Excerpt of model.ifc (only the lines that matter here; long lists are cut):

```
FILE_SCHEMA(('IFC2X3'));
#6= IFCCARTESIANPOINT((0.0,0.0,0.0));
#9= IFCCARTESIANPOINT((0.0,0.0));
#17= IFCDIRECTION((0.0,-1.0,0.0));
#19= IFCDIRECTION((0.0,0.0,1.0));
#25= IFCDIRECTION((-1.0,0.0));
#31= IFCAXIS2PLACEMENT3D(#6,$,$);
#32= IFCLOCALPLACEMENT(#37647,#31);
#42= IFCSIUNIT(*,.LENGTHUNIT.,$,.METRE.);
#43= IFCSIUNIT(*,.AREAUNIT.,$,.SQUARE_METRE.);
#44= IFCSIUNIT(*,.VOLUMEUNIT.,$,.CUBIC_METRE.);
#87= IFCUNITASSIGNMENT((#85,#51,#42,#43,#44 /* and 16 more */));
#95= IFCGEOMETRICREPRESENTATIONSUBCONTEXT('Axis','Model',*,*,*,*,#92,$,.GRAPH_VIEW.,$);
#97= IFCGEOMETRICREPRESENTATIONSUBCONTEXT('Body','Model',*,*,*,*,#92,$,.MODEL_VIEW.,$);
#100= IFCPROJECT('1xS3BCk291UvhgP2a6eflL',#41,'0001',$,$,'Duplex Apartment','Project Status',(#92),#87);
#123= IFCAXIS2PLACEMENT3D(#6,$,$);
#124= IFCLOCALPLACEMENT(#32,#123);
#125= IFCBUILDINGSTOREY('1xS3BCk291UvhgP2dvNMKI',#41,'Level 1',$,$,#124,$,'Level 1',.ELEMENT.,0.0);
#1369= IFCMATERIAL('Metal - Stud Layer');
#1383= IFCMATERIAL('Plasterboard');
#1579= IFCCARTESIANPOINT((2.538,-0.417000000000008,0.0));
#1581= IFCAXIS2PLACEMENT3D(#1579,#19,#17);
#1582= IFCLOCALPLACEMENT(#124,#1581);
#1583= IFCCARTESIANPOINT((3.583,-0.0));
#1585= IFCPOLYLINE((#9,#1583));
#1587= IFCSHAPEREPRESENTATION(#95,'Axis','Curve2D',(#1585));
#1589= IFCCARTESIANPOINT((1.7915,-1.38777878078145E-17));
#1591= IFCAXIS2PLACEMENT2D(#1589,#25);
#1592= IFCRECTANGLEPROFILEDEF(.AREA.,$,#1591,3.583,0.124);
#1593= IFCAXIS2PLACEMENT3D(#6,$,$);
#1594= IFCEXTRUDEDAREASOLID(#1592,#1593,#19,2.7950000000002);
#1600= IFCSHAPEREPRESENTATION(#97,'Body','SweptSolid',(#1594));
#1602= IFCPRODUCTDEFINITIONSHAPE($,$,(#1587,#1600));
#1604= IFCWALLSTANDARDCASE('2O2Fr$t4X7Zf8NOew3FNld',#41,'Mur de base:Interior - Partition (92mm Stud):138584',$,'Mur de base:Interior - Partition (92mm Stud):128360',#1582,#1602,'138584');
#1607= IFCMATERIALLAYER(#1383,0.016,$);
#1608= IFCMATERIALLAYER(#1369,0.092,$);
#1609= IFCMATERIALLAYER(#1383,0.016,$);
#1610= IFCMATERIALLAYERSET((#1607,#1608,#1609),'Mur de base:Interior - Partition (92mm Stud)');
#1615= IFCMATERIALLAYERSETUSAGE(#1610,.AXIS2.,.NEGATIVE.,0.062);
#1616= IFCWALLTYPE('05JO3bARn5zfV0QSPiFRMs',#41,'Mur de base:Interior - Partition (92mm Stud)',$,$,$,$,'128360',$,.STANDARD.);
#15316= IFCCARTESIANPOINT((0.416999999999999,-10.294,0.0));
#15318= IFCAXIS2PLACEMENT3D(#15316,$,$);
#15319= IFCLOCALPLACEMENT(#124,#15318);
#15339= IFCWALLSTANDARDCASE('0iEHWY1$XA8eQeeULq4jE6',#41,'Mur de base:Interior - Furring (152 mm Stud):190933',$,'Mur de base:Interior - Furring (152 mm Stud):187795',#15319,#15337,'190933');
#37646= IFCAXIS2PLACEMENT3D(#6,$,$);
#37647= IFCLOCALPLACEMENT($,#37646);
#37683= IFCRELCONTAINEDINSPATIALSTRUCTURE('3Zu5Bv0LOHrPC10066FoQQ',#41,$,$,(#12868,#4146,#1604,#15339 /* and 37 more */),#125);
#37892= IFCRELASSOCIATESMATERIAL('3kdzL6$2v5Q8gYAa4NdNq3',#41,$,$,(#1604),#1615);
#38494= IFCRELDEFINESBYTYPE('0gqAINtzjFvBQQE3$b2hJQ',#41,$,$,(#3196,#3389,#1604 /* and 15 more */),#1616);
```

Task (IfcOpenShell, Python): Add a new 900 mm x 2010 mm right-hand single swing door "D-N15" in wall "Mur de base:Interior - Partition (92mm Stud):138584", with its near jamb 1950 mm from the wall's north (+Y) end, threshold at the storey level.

```python
import numpy as np
import ifcopenshell
import ifcopenshell.api.feature
import ifcopenshell.api.geometry
import ifcopenshell.api.root
import ifcopenshell.api.spatial
import ifcopenshell.api.type
import ifcopenshell.geom
import ifcopenshell.util.element
import ifcopenshell.util.placement
import ifcopenshell.util.representation
import ifcopenshell.util.shape
import ifcopenshell.util.unit

model = ifcopenshell.open("model.ifc")
unit_scale = ifcopenshell.util.unit.calculate_unit_scale(model)
settings = ifcopenshell.geom.settings()


def volume(element):
    """Net volume in cubic metres, openings subtracted."""
    shape = ifcopenshell.geom.create_shape(settings, element)
    return ifcopenshell.util.shape.get_volume(shape.geometry)


wall = model.by_guid("2O2Fr$t4X7Zf8NOew3FNld")
storey = ifcopenshell.util.element.get_container(wall, ifc_class="IfcBuildingStorey")
context = ifcopenshell.util.representation.get_context(model, "Model", "Body", "MODEL_VIEW")
before = volume(wall)

width, height, from_end, sill = 0.9, 2.01, 1.95, 0.0  # metres

# The wall runs along its own X axis, and the end named is its -X end.
wall_shape = ifcopenshell.geom.create_shape(settings, wall)
x, y, z = ifcopenshell.util.shape.get_vertices(wall_shape.geometry).T
start = x.min() + from_end
face, thickness = float(y.min()), float(y.max() - y.min())
wall_matrix = ifcopenshell.util.placement.get_local_placement(wall.ObjectPlacement)
level = ifcopenshell.util.placement.get_local_placement(storey.ObjectPlacement)[2, 3]


def in_wall(x, y):
    """Placement at x, y metres in the wall's axes, at sill height."""
    matrix = wall_matrix.copy()
    matrix[:, 3] = wall_matrix @ np.array([x / unit_scale, y / unit_scale, 0.0, 1.0])
    matrix[2, 3] = level + sill / unit_scale
    return matrix


# Opening: a box that overshoots both wall faces by 50 mm.
opening = ifcopenshell.api.root.create_entity(model, ifc_class="IfcOpeningElement")
box = ifcopenshell.api.geometry.add_wall_representation(
    model, context=context, length=width, height=height, thickness=thickness + 0.1
)
ifcopenshell.api.geometry.assign_representation(model, product=opening, representation=box)
ifcopenshell.api.geometry.edit_object_placement(model, product=opening, matrix=in_wall(start, face - 0.05), is_si=False)
ifcopenshell.api.feature.add_feature(model, feature=opening, element=wall)

door = ifcopenshell.api.root.create_entity(model, ifc_class="IfcDoor", name="D-N15")
door.OverallWidth, door.OverallHeight = width / unit_scale, height / unit_scale
body = ifcopenshell.api.geometry.add_door_representation(
    model,
    context=context,
    overall_width=door.OverallWidth,
    overall_height=door.OverallHeight,
    operation_type="SINGLE_SWING_RIGHT",
    lining_properties={"LiningDepth": thickness / unit_scale, "ThresholdDepth": thickness / unit_scale},
)
ifcopenshell.api.geometry.assign_representation(model, product=door, representation=body)
ifcopenshell.api.spatial.assign_container(model, products=[door], relating_structure=storey)
fills = ifcopenshell.api.feature.add_filling(model, opening=opening, element=door)
fills.OwnerHistory = door.OwnerHistory  # required in IFC2X3

# IFC2X3 keeps the operation on the door style.
style = ifcopenshell.api.root.create_entity(model, ifc_class="IfcDoorStyle", name="D-N15")
style.OperationType, style.ConstructionType = "SINGLE_SWING_RIGHT", "NOTDEFINED"
style.ParameterTakesPrecedence = style.Sizeable = False
ifcopenshell.api.type.assign_type(model, related_objects=[door], relating_type=style)

# The lining spans the wall, so the door starts at the wall face.
ifcopenshell.api.geometry.edit_object_placement(model, product=door, matrix=in_wall(start, face), is_si=False)

after = volume(wall)

print(f"wall volume {before:.3f} -> {after:.3f} m3")

model.write("model_v2.ifc")
```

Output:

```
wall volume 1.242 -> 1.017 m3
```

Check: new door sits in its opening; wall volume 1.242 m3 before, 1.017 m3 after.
